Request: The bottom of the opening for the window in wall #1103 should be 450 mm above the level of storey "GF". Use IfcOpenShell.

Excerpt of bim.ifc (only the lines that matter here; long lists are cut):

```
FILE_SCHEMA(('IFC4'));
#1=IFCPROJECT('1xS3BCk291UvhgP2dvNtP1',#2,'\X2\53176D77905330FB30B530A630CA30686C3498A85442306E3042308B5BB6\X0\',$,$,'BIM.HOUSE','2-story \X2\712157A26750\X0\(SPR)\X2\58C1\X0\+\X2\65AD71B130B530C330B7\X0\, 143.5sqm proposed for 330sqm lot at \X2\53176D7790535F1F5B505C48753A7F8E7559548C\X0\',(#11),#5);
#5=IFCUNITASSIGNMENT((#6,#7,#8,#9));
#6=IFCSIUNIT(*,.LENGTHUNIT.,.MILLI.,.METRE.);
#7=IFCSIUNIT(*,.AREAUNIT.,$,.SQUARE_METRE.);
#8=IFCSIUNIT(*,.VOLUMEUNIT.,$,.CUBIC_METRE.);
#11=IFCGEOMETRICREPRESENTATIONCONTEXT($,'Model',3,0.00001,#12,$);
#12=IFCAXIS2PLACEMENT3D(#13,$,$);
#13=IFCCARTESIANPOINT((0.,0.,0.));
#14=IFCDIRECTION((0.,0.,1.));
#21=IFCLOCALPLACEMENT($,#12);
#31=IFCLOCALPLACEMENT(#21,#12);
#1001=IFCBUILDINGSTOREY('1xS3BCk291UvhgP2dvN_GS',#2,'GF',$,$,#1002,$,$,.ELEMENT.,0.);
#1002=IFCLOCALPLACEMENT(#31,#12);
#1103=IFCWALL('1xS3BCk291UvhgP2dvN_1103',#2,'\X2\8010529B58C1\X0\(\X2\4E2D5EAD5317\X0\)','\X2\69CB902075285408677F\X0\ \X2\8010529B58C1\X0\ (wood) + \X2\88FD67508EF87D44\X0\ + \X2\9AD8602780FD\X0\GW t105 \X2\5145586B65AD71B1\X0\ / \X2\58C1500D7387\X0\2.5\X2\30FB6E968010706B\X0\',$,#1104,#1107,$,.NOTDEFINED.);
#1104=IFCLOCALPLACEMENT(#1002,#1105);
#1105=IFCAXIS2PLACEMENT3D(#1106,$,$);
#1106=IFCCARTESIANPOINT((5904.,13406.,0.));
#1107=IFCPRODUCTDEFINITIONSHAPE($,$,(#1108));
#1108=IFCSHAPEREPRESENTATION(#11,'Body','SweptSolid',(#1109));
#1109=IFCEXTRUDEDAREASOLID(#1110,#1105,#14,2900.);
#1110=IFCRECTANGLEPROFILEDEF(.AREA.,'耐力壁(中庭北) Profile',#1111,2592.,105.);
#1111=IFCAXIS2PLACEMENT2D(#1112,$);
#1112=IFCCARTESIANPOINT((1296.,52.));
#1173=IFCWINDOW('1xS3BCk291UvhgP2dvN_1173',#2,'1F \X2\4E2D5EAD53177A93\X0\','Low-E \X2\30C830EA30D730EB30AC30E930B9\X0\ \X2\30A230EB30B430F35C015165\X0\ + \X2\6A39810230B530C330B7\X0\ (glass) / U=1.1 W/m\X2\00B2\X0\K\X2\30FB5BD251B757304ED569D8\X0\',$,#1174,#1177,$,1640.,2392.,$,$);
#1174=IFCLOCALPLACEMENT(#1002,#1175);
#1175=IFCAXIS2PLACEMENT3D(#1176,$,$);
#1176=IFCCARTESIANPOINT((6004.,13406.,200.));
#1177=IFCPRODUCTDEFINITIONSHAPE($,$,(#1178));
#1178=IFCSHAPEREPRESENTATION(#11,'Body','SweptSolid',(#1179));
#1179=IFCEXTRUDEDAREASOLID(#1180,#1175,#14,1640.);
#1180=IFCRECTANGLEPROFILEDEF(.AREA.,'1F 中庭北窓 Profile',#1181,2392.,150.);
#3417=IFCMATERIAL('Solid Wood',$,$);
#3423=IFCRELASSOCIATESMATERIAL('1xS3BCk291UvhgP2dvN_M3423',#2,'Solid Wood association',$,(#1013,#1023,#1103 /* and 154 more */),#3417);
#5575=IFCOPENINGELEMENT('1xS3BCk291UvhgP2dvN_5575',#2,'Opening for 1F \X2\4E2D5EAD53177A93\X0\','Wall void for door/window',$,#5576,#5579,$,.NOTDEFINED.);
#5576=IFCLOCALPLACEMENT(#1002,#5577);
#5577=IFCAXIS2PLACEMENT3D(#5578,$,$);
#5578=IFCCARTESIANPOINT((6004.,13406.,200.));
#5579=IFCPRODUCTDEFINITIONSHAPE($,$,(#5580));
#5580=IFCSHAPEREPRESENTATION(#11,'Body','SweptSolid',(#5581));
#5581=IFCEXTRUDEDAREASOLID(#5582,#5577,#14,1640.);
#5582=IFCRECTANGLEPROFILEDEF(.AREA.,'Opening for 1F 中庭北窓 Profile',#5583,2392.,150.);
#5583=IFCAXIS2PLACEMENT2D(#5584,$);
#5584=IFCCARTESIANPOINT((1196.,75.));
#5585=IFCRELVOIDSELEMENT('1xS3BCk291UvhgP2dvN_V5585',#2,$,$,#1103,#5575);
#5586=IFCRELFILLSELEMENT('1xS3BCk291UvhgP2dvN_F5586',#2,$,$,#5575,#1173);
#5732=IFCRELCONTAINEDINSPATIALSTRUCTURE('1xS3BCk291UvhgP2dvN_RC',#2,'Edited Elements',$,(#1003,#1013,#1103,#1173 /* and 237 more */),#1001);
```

```python
import numpy as np
import ifcopenshell
import ifcopenshell.api.geometry
import ifcopenshell.geom
import ifcopenshell.util.element
import ifcopenshell.util.placement
import ifcopenshell.util.shape
import ifcopenshell.util.unit

model = ifcopenshell.open("bim.ifc")
unit_scale = ifcopenshell.util.unit.calculate_unit_scale(model)

window = model.by_guid("1xS3BCk291UvhgP2dvN_1173")
opening = window.FillsVoids[0].RelatingOpeningElement
storey = ifcopenshell.util.element.get_container(window, ifc_class="IfcBuildingStorey")
level = ifcopenshell.util.placement.get_local_placement(storey.ObjectPlacement)[2, 3]

# The opening's origin need not be at the sill, so measure its lowest point.
shape = ifcopenshell.geom.create_shape(ifcopenshell.geom.settings(), opening)
bottom = ifcopenshell.util.shape.get_shape_bottom_elevation(shape, shape.geometry) / unit_scale
dz = level + 0.45 / unit_scale - bottom

shift = np.array([0.0, 0.0, dz])
# The window is not placed relative to its opening, so move both.
for product in (opening, window):
    matrix = ifcopenshell.util.placement.get_local_placement(product.ObjectPlacement)
    matrix[:3, 3] += shift
    ifcopenshell.api.geometry.edit_object_placement(model, product=product, matrix=matrix, is_si=False)

print(f"moved by {dz * unit_scale:+.3f} m")

model.write("bim_edited.ifc")
```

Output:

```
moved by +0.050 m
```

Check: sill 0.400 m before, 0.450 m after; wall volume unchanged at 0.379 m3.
